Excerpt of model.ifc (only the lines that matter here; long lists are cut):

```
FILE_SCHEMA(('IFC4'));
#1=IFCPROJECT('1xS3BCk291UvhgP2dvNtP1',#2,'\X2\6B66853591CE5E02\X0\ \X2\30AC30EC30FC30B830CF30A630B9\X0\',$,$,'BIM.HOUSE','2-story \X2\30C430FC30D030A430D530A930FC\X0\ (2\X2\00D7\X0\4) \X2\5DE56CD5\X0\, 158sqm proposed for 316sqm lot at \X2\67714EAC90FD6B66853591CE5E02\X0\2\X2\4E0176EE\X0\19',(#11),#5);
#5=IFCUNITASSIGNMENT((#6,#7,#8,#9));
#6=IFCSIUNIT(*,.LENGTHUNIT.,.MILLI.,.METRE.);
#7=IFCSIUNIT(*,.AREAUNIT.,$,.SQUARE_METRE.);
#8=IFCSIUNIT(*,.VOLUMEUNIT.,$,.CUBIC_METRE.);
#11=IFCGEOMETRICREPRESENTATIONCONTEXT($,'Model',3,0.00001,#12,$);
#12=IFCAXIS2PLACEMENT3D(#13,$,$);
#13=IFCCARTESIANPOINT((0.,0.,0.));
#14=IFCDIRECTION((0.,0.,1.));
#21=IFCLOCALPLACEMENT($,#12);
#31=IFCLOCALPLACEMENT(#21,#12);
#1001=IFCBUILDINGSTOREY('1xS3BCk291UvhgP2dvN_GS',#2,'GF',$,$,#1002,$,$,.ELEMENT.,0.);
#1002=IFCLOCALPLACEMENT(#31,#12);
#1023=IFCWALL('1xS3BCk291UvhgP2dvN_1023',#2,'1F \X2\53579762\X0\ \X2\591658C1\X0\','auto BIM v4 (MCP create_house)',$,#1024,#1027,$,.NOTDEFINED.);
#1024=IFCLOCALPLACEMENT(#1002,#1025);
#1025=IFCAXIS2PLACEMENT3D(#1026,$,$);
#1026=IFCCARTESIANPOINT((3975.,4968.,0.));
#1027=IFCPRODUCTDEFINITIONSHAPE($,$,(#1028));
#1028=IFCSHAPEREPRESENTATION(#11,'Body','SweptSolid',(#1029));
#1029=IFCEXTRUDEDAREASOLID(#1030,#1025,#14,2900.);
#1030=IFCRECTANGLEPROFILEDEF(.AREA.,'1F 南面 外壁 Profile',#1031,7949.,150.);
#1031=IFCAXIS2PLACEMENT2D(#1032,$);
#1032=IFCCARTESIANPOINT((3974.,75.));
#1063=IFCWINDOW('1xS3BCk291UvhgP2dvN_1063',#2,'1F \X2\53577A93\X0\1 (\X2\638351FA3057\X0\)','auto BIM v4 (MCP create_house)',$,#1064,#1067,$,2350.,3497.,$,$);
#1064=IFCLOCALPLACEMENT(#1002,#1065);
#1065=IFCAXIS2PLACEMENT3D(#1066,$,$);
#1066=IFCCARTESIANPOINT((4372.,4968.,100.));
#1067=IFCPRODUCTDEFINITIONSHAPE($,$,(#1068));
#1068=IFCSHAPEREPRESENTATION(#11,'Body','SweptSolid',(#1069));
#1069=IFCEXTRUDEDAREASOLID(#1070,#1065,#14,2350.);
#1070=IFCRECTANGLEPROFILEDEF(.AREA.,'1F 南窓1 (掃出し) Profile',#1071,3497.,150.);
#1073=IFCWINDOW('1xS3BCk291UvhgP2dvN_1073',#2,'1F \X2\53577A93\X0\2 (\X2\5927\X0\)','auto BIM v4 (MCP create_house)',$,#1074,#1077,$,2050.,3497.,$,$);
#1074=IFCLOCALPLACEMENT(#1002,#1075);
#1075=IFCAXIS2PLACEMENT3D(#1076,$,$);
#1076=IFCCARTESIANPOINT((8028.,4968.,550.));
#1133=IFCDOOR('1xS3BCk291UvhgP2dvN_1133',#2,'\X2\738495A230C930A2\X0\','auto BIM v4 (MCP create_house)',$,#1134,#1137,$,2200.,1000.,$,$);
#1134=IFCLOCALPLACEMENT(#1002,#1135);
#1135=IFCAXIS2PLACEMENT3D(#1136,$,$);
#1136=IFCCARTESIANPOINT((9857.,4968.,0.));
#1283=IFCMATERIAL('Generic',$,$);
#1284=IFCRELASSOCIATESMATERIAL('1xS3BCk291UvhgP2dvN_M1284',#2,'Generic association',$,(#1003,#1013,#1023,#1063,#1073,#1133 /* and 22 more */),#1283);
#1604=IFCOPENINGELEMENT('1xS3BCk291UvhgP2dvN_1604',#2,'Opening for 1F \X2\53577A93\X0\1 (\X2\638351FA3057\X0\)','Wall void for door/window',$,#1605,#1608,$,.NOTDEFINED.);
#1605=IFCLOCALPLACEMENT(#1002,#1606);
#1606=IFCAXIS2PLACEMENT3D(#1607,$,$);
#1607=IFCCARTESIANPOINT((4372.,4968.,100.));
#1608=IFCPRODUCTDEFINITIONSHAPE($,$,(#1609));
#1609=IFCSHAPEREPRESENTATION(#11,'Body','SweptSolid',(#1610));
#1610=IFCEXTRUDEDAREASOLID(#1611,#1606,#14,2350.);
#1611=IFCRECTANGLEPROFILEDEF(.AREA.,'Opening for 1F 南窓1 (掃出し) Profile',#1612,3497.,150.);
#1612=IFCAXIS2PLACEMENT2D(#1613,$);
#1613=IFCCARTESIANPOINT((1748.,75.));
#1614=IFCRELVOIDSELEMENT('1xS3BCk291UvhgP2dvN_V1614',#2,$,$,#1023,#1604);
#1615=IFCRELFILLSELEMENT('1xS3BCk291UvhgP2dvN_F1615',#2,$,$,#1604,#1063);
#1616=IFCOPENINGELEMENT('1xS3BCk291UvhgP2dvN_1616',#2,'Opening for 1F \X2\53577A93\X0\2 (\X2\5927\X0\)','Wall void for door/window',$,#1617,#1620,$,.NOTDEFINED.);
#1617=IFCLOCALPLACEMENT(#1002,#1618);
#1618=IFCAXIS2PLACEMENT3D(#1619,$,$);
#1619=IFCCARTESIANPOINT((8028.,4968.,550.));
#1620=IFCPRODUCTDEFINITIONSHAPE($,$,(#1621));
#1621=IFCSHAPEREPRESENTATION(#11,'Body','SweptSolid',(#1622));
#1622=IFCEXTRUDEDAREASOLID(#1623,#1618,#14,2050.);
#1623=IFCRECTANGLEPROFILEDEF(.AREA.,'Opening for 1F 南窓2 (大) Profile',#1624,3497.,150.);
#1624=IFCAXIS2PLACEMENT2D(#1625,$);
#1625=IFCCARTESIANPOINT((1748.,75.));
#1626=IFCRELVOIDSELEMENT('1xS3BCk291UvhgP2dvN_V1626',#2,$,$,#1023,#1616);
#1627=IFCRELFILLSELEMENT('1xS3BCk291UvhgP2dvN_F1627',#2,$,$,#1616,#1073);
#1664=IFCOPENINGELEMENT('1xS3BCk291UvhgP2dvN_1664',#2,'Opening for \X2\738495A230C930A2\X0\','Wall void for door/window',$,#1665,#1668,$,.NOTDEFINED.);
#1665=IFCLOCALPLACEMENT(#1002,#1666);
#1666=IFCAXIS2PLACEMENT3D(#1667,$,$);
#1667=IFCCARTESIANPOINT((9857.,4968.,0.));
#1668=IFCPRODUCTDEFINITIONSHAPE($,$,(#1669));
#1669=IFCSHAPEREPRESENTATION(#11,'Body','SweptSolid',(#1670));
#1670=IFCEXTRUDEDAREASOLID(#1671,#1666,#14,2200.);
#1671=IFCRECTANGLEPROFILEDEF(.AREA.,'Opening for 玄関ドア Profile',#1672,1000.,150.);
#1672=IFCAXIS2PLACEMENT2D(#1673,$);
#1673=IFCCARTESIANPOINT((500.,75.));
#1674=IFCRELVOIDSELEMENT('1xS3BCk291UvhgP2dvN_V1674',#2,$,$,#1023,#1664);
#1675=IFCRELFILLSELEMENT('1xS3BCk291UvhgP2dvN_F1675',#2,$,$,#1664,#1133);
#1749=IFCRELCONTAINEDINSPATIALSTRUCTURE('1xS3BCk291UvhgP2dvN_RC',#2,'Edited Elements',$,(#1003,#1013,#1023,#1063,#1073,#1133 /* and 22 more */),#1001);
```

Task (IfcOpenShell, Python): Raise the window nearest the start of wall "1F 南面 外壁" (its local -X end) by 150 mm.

```python
import numpy as np
import ifcopenshell
import ifcopenshell.api.geometry
import ifcopenshell.util.placement
import ifcopenshell.util.unit

model = ifcopenshell.open("model.ifc")
unit_scale = ifcopenshell.util.unit.calculate_unit_scale(model)

window = model.by_id(1063)
opening = window.FillsVoids[0].RelatingOpeningElement
dz = 0.15 / unit_scale

shift = np.array([0.0, 0.0, dz])
# The window is not placed relative to its opening, so move both.
for product in (opening, window):
    matrix = ifcopenshell.util.placement.get_local_placement(product.ObjectPlacement)
    matrix[:3, 3] += shift
    ifcopenshell.api.geometry.edit_object_placement(model, product=product, matrix=matrix, is_si=False)

print(f"moved by {dz * unit_scale:+.3f} m")

model.write("model_edited.ifc")
```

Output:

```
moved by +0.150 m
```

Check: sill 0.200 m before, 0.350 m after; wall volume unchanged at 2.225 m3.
